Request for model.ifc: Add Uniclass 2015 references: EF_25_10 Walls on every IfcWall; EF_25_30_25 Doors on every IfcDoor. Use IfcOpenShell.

First a look at what the model holds.

```python
import ifcopenshell

model = ifcopenshell.open("model.ifc")
print(model.schema)
print("classifications:", [c.Name for c in model.by_type("IfcClassification")])
for ifc_class in ("IfcDoor", "IfcRoof", "IfcStair", "IfcWall", "IfcWindow"):
    print(ifc_class, len(model.by_type(ifc_class)))
```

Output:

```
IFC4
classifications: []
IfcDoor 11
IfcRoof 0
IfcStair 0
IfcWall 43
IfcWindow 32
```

```python
import ifcopenshell
import ifcopenshell.api.classification

model = ifcopenshell.open("model.ifc")

system = ifcopenshell.api.classification.add_classification(model, classification="Uniclass 2015")

codes = {
    "IfcWall": ("EF_25_10", "Walls"),
    "IfcDoor": ("EF_25_30_25", "Doors"),
}
for ifc_class, (code, name) in codes.items():
    products = model.by_type(ifc_class)
    ifcopenshell.api.classification.add_reference(
        model, products=products, classification=system, identification=code, name=name
    )
    print(code, len(products))

model.write("model_rev.ifc")
```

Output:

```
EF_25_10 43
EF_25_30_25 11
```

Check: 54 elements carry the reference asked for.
